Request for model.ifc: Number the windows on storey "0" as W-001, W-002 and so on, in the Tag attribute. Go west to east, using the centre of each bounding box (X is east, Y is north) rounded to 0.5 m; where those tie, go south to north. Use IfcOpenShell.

First a look at what the model holds.

```python
import ifcopenshell
import ifcopenshell.util.element
import ifcopenshell.util.placement

model = ifcopenshell.open("model.ifc")
print(model.schema)
storey = next(s for s in model.by_type("IfcBuildingStorey") if s.Name == "0")
windows = [e for e in ifcopenshell.util.element.get_decomposition(storey) if e.is_a("IfcWindow")]
for e in sorted(windows, key=lambda e: e.id()):
    origin = ifcopenshell.util.placement.get_local_placement(e.ObjectPlacement)[:3, 3]
    print(e.id(), e.Tag, e.Name, origin.round(2) + 0.0, sep=" | ")
```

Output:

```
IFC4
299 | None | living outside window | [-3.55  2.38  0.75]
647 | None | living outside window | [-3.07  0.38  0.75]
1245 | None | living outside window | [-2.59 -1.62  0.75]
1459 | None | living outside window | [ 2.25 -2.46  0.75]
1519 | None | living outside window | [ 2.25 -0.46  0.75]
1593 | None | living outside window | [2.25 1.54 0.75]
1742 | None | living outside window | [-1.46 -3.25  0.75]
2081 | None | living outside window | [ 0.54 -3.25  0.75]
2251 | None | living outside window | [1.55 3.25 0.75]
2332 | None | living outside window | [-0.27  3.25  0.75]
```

```python
import ifcopenshell
import ifcopenshell.geom
import ifcopenshell.util.element
import ifcopenshell.util.shape

model = ifcopenshell.open("model.ifc")
settings = ifcopenshell.geom.settings()
settings.set("use-world-coords", True)


def centre(element):
    shape = ifcopenshell.geom.create_shape(settings, element)
    return ifcopenshell.util.shape.get_bbox_centroid(shape.geometry)


storey = next(s for s in model.by_type("IfcBuildingStorey") if s.Name == "0")
windows = [e for e in ifcopenshell.util.element.get_decomposition(storey) if e.is_a("IfcWindow")]

# Insertion points can sit at a corner or the storey origin, so sort by the geometry (in metres).
centres = {e: centre(e) for e in windows}
windows.sort(key=lambda e: (round(centres[e][0] / 0.5), centres[e][1]))

for i, e in enumerate(windows, start=1):
    number = f"W-0{i:02d}"
    e.Tag = number
    print(e.id(), number)

model.write("model-out.ifc")
```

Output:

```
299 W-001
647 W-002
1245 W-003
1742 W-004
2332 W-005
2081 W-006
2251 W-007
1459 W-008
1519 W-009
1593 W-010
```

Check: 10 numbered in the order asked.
